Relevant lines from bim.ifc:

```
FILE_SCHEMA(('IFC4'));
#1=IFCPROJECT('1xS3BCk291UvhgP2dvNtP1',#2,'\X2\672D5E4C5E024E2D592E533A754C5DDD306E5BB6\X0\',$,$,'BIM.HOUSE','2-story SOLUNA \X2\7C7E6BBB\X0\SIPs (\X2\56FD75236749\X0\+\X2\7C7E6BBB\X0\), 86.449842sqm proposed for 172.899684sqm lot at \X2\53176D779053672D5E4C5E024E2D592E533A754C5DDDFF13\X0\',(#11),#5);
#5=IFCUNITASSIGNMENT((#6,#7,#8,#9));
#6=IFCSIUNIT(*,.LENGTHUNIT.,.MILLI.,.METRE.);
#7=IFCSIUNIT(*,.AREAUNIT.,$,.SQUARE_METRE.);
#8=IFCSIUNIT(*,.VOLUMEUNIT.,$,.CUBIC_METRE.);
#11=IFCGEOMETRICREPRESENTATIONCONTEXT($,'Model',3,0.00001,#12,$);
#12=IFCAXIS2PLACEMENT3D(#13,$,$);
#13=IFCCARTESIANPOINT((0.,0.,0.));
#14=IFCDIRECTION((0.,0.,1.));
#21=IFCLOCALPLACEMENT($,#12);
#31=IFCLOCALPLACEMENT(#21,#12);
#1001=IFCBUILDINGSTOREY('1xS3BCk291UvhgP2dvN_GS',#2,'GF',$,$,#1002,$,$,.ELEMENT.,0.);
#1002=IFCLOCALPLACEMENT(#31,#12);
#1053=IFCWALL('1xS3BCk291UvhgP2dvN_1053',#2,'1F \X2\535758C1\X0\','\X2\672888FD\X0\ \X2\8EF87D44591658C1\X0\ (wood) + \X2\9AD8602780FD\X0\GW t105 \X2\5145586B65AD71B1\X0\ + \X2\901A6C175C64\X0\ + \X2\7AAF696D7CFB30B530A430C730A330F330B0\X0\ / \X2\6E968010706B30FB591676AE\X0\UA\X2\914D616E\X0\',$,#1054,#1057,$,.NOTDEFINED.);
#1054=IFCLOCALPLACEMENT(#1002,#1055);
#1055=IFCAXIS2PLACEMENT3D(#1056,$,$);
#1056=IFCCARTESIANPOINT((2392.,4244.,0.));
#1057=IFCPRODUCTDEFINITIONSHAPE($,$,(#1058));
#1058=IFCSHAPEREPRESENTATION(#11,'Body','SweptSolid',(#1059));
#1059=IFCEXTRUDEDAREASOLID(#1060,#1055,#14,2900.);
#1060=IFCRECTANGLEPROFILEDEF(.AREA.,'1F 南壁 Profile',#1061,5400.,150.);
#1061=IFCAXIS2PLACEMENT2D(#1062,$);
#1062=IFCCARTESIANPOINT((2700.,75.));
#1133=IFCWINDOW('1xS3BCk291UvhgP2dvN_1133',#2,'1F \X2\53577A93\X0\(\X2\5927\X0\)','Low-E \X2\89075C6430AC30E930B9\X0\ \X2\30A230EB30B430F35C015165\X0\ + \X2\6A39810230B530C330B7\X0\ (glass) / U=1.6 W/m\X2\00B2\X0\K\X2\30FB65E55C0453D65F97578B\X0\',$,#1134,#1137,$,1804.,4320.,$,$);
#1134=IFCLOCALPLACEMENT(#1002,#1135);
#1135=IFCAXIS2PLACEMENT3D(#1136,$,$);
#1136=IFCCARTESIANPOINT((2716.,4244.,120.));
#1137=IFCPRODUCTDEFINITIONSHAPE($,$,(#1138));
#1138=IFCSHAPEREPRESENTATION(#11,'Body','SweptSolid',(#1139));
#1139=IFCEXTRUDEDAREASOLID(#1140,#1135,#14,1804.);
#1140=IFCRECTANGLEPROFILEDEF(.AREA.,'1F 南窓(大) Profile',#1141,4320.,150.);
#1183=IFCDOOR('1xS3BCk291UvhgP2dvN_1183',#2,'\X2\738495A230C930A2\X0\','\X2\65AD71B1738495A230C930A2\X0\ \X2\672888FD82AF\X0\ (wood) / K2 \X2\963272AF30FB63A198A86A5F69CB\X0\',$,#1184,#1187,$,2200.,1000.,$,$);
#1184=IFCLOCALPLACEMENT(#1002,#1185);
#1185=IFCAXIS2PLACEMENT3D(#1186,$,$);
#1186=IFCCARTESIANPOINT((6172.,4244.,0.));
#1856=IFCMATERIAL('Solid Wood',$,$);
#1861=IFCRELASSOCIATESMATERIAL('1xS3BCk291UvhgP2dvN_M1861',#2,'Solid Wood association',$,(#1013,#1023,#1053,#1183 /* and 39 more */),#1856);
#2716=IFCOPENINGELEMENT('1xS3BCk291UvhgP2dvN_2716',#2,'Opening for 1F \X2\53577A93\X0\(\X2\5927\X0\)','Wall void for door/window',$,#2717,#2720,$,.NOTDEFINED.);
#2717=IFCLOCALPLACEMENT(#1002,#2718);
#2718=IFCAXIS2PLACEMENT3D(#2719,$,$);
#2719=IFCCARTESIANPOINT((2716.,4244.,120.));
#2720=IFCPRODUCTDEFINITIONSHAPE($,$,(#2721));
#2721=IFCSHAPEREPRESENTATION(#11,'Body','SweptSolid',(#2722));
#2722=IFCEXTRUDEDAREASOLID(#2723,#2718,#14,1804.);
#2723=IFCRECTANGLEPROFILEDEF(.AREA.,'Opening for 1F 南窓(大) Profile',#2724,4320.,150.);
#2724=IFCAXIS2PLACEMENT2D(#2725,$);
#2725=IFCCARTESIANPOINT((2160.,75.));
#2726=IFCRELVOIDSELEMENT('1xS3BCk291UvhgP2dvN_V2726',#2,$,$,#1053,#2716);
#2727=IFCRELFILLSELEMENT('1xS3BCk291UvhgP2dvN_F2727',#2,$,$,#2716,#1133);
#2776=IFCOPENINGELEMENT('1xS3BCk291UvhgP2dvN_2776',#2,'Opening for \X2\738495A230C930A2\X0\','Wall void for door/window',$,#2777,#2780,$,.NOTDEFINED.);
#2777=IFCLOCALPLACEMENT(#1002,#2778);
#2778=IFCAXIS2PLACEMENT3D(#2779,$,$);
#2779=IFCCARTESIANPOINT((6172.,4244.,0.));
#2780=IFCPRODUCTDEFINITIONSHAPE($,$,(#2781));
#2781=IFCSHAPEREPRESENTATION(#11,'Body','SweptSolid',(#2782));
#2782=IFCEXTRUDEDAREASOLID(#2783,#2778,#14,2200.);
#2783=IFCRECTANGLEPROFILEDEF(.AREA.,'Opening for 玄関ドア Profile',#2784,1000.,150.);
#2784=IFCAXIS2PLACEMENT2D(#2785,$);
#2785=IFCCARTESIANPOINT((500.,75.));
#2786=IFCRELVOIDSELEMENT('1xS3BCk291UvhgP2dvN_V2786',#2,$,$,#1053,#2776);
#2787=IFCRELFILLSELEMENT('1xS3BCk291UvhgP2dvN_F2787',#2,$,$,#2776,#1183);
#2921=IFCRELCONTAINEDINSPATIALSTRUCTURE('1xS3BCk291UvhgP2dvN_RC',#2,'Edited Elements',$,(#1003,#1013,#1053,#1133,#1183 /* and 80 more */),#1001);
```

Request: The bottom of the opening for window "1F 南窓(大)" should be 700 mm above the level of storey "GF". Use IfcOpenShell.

```python
import numpy as np
import ifcopenshell
import ifcopenshell.api.geometry
import ifcopenshell.geom
import ifcopenshell.util.element
import ifcopenshell.util.placement
import ifcopenshell.util.shape
import ifcopenshell.util.unit

model = ifcopenshell.open("bim.ifc")
unit_scale = ifcopenshell.util.unit.calculate_unit_scale(model)

window = model.by_guid("1xS3BCk291UvhgP2dvN_1133")
opening = window.FillsVoids[0].RelatingOpeningElement
storey = ifcopenshell.util.element.get_container(window, ifc_class="IfcBuildingStorey")
level = ifcopenshell.util.placement.get_local_placement(storey.ObjectPlacement)[2, 3]

# The opening's origin need not be at the sill, so measure its lowest point.
shape = ifcopenshell.geom.create_shape(ifcopenshell.geom.settings(), opening)
bottom = ifcopenshell.util.shape.get_shape_bottom_elevation(shape, shape.geometry) / unit_scale
dz = level + 0.7 / unit_scale - bottom

shift = np.array([0.0, 0.0, dz])
# The window is not placed relative to its opening, so move both.
for product in (opening, window):
    matrix = ifcopenshell.util.placement.get_local_placement(product.ObjectPlacement)
    matrix[:3, 3] += shift
    ifcopenshell.api.geometry.edit_object_placement(model, product=product, matrix=matrix, is_si=False)

print(f"moved by {dz * unit_scale:+.3f} m")

model.write("bim_v2.ifc")
```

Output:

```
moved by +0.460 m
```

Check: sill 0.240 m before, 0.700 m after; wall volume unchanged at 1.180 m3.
